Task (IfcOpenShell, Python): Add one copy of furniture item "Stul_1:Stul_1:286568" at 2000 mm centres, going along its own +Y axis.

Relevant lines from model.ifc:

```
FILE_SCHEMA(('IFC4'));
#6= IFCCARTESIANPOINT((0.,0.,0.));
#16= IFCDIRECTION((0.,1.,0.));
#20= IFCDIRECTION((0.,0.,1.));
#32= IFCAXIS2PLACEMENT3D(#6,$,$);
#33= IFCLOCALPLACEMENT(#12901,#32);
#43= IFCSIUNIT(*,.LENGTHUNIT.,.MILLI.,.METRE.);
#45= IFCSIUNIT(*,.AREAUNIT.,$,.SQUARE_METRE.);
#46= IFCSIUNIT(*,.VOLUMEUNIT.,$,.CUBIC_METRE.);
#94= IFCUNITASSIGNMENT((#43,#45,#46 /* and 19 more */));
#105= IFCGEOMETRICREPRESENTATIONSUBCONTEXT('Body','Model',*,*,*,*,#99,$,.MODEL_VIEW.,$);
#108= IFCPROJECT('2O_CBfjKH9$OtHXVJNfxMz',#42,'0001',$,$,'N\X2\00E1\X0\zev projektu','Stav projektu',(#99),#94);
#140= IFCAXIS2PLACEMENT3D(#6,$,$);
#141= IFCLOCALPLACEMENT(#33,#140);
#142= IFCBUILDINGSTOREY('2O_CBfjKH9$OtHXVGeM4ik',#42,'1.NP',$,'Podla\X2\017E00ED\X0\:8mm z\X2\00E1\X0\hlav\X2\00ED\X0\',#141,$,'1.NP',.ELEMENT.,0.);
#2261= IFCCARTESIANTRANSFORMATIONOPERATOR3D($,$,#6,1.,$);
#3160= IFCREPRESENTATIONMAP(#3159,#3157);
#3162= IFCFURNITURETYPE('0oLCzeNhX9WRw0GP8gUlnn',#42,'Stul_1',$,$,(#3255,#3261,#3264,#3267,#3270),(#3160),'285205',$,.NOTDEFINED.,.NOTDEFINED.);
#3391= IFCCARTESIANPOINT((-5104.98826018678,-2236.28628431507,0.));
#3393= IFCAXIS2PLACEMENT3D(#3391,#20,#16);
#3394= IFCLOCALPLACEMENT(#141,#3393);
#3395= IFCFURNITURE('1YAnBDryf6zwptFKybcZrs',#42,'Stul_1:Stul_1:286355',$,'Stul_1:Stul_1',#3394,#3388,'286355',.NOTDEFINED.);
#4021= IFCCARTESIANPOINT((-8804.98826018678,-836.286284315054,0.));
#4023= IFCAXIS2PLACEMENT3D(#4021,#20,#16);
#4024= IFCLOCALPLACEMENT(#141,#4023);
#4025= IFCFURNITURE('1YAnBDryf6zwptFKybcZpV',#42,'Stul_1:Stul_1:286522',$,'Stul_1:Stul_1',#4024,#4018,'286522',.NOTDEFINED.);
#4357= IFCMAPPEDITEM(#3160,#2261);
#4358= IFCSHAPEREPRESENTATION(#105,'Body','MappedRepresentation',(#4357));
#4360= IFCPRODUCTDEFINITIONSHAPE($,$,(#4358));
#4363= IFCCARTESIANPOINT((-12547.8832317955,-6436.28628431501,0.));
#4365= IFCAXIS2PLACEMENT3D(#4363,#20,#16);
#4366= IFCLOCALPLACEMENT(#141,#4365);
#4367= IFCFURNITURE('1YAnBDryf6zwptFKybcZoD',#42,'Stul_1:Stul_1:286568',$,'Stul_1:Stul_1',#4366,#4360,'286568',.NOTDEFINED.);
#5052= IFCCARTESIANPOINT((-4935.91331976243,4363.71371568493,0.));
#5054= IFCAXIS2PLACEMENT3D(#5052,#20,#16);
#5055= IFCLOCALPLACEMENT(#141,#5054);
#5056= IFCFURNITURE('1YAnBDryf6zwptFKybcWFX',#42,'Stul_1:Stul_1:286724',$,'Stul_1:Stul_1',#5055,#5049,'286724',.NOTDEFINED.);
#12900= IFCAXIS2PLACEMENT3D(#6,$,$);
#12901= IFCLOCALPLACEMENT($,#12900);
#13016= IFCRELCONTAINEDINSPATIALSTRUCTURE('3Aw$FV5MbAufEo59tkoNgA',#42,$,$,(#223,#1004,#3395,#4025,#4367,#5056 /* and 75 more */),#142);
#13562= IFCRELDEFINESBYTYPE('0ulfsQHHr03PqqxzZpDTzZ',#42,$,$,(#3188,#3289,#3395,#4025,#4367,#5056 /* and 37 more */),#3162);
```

```python
import ifcopenshell
import ifcopenshell.api.geometry
import ifcopenshell.api.root
import ifcopenshell.util.element
import ifcopenshell.util.placement
import ifcopenshell.util.unit

model = ifcopenshell.open("model.ifc")
unit_scale = ifcopenshell.util.unit.calculate_unit_scale(model)


def reuse_history(source, copy):
    """copy_class also copies each property set's owner history, people and application; keep the originals."""
    for rel in copy.IsDefinedBy:
        if rel.is_a("IfcRelDefinesByProperties") and (history := rel.RelatingPropertyDefinition.OwnerHistory):
            rel.RelatingPropertyDefinition.OwnerHistory = source.OwnerHistory
            ifcopenshell.util.element.remove_deep2(model, history)


source = model.by_guid("1YAnBDryf6zwptFKybcZoD")
base = ifcopenshell.util.placement.get_local_placement(source.ObjectPlacement)
step = base[:3, 1] * 2 / unit_scale

for i in range(1, 2):
    copy = ifcopenshell.api.root.copy_class(model, product=source)
    copy.Representation = ifcopenshell.util.element.copy_deep(
        model, source.Representation, exclude=["IfcGeometricRepresentationContext", "IfcRepresentationMap"]
    )
    copy.Name = "Stul_1:Stul_1"
    copy.Tag = None
    reuse_history(source, copy)
    matrix = base.copy()
    matrix[:3, 3] += i * step
    print("added at", matrix[:3, 3].round(3) + 0.0)
    ifcopenshell.api.geometry.edit_object_placement(model, product=copy, matrix=matrix, is_si=False)

model.write("model-out.ifc")
```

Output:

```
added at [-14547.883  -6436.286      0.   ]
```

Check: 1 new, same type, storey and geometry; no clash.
